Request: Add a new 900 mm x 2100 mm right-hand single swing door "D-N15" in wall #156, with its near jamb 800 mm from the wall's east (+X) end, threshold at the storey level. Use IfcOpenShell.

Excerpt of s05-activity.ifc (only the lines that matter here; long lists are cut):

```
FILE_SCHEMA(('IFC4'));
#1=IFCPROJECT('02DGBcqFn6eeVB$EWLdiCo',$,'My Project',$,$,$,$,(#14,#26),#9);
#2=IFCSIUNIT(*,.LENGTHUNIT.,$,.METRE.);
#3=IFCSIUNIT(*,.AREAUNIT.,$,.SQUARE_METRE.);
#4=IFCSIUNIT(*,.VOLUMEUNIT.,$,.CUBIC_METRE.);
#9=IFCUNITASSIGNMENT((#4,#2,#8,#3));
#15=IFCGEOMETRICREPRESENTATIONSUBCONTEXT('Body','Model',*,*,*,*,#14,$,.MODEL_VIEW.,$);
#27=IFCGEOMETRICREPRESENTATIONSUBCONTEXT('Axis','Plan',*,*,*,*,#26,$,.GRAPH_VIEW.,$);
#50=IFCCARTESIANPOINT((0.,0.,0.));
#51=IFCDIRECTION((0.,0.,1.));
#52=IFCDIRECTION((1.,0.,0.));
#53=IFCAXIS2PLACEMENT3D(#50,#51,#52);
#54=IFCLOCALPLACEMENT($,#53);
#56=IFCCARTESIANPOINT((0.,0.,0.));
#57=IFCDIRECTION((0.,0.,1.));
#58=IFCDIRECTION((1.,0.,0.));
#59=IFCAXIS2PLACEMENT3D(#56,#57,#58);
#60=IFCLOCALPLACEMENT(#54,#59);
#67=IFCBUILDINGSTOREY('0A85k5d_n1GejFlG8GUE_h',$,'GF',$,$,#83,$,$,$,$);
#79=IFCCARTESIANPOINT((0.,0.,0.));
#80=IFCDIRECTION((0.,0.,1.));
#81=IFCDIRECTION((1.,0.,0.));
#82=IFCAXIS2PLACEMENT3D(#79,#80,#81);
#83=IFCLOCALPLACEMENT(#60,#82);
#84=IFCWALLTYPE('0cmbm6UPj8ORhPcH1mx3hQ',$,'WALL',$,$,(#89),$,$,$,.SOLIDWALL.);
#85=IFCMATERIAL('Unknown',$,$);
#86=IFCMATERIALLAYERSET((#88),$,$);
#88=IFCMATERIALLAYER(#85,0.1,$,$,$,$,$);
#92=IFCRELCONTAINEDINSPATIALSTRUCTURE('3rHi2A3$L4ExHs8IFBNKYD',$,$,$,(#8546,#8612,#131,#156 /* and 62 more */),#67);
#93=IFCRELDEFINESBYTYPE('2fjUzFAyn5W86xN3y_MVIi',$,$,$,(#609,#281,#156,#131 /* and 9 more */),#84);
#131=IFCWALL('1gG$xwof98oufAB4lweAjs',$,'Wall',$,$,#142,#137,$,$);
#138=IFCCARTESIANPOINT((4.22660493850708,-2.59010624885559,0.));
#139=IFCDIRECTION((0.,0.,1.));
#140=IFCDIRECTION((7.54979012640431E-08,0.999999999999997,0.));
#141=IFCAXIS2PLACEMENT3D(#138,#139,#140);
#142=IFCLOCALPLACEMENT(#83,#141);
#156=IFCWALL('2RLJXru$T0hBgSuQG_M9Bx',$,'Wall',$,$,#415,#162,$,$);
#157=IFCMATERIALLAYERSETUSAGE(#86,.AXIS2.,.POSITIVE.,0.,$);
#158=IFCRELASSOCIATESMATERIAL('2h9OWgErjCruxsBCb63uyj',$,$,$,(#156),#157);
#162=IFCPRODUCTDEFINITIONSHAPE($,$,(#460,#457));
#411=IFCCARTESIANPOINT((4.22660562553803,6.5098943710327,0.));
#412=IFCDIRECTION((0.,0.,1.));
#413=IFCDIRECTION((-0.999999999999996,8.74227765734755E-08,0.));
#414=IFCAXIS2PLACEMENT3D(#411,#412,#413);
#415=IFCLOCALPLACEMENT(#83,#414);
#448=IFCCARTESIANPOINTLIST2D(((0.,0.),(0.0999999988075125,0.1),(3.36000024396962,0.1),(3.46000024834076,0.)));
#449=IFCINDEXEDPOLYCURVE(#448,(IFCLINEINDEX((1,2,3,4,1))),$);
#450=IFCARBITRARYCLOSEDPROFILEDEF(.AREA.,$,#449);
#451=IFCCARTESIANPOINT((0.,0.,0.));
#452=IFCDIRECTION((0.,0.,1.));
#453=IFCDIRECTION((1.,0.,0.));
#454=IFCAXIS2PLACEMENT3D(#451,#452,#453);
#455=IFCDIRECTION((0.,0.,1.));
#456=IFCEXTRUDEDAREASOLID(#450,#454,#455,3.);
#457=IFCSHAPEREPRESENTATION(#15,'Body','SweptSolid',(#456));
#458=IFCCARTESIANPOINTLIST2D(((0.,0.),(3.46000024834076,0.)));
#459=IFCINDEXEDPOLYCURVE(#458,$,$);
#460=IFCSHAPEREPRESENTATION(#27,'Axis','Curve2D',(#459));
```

```python
import numpy as np
import ifcopenshell
import ifcopenshell.api.feature
import ifcopenshell.api.geometry
import ifcopenshell.api.root
import ifcopenshell.api.spatial
import ifcopenshell.geom
import ifcopenshell.util.element
import ifcopenshell.util.placement
import ifcopenshell.util.representation
import ifcopenshell.util.shape
import ifcopenshell.util.unit

model = ifcopenshell.open("s05-activity.ifc")
unit_scale = ifcopenshell.util.unit.calculate_unit_scale(model)
settings = ifcopenshell.geom.settings()


def volume(element):
    """Net volume in cubic metres, openings subtracted."""
    shape = ifcopenshell.geom.create_shape(settings, element)
    return ifcopenshell.util.shape.get_volume(shape.geometry)


wall = model.by_id(156)
storey = ifcopenshell.util.element.get_container(wall, ifc_class="IfcBuildingStorey")
context = ifcopenshell.util.representation.get_context(model, "Model", "Body", "MODEL_VIEW")
before = volume(wall)

width, height, from_end, sill = 0.9, 2.1, 0.8, 0.0  # metres

# The wall runs along its own X axis, and the end named is its -X end.
wall_shape = ifcopenshell.geom.create_shape(settings, wall)
x, y, z = ifcopenshell.util.shape.get_vertices(wall_shape.geometry).T
start = x.min() + from_end
face, thickness = float(y.min()), float(y.max() - y.min())
wall_matrix = ifcopenshell.util.placement.get_local_placement(wall.ObjectPlacement)
level = ifcopenshell.util.placement.get_local_placement(storey.ObjectPlacement)[2, 3]


def in_wall(x, y):
    """Placement at x, y metres in the wall's axes, at sill height."""
    matrix = wall_matrix.copy()
    matrix[:, 3] = wall_matrix @ np.array([x / unit_scale, y / unit_scale, 0.0, 1.0])
    matrix[2, 3] = level + sill / unit_scale
    return matrix


# Opening: a box that overshoots both wall faces by 50 mm.
opening = ifcopenshell.api.root.create_entity(model, ifc_class="IfcOpeningElement", predefined_type="OPENING")
box = ifcopenshell.api.geometry.add_wall_representation(
    model, context=context, length=width, height=height, thickness=thickness + 0.1
)
ifcopenshell.api.geometry.assign_representation(model, product=opening, representation=box)
ifcopenshell.api.geometry.edit_object_placement(model, product=opening, matrix=in_wall(start, face - 0.05), is_si=False)
ifcopenshell.api.feature.add_feature(model, feature=opening, element=wall)

door = ifcopenshell.api.root.create_entity(model, ifc_class="IfcDoor", name="D-N15", predefined_type="DOOR")
door.OverallWidth, door.OverallHeight = width / unit_scale, height / unit_scale
door.OperationType = "SINGLE_SWING_RIGHT"
body = ifcopenshell.api.geometry.add_door_representation(
    model,
    context=context,
    overall_width=door.OverallWidth,
    overall_height=door.OverallHeight,
    operation_type="SINGLE_SWING_RIGHT",
    lining_properties={"LiningDepth": thickness / unit_scale, "ThresholdDepth": thickness / unit_scale},
)
ifcopenshell.api.geometry.assign_representation(model, product=door, representation=body)
ifcopenshell.api.spatial.assign_container(model, products=[door], relating_structure=storey)
ifcopenshell.api.feature.add_filling(model, opening=opening, element=door)

# The lining spans the wall, so the door starts at the wall face.
ifcopenshell.api.geometry.edit_object_placement(model, product=door, matrix=in_wall(start, face), is_si=False)

after = volume(wall)

print(f"wall volume {before:.3f} -> {after:.3f} m3")

model.write("s05-activity_v2.ifc")
```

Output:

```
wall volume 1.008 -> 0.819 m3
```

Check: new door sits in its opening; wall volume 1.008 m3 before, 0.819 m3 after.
